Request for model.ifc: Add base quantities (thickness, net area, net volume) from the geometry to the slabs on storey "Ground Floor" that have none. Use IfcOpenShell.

First a look at what the model holds.

```python
import ifcopenshell
import ifcopenshell.util.element
import ifcopenshell.util.unit

model = ifcopenshell.open("model.ifc")
print(model.schema)
for unit_type in ("LENGTHUNIT", "AREAUNIT", "VOLUMEUNIT"):
    print(unit_type, ifcopenshell.util.unit.calculate_unit_scale(model, unit_type))
storey = next(s for s in model.by_type("IfcBuildingStorey") if s.Name == "Ground Floor")
slabs = [e for e in ifcopenshell.util.element.get_decomposition(storey) if e.is_a("IfcSlab")]
for e in sorted(slabs, key=lambda e: e.id()):
    print(e.id(), e.is_a(), e.Name, list(ifcopenshell.util.element.get_psets(e, qtos_only=True)), sep=" | ")
```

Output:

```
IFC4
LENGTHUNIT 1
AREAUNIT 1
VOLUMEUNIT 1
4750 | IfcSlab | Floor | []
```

```python
import ifcopenshell
import ifcopenshell.api.pset
import ifcopenshell.geom
import ifcopenshell.util.element
import ifcopenshell.util.shape
import ifcopenshell.util.unit

model = ifcopenshell.open("model.ifc")
unit_scale = ifcopenshell.util.unit.calculate_unit_scale(model)
area_scale = ifcopenshell.util.unit.calculate_unit_scale(model, "AREAUNIT")
volume_scale = ifcopenshell.util.unit.calculate_unit_scale(model, "VOLUMEUNIT")
settings = ifcopenshell.geom.settings()

storey = next(s for s in model.by_type("IfcBuildingStorey") if s.Name == "Ground Floor")
slabs = [e for e in ifcopenshell.util.element.get_decomposition(storey) if e.is_a("IfcSlab")]

for e in sorted(slabs, key=lambda e: e.id()):
    if ifcopenshell.util.element.get_psets(e, qtos_only=True, should_inherit=False):
        continue
    # Geometry comes back in metres, in the element's own axes.
    shape = ifcopenshell.geom.create_shape(settings, e)
    values = {
        "Width": ifcopenshell.util.shape.get_z(shape.geometry) / unit_scale,
        "NetArea": ifcopenshell.util.shape.get_footprint_area(shape.geometry) / area_scale,
        "NetVolume": ifcopenshell.util.shape.get_volume(shape.geometry) / volume_scale,
    }
    qto = ifcopenshell.api.pset.add_qto(model, product=e, name="Qto_SlabBaseQuantities")
    ifcopenshell.api.pset.edit_qto(model, qto=qto, properties=values)
    print(e.id(), {k: round(v, 3) for k, v in values.items()})

model.write("model_v2.ifc")
```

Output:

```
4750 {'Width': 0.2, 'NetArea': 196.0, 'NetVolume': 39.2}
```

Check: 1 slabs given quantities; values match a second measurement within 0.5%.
